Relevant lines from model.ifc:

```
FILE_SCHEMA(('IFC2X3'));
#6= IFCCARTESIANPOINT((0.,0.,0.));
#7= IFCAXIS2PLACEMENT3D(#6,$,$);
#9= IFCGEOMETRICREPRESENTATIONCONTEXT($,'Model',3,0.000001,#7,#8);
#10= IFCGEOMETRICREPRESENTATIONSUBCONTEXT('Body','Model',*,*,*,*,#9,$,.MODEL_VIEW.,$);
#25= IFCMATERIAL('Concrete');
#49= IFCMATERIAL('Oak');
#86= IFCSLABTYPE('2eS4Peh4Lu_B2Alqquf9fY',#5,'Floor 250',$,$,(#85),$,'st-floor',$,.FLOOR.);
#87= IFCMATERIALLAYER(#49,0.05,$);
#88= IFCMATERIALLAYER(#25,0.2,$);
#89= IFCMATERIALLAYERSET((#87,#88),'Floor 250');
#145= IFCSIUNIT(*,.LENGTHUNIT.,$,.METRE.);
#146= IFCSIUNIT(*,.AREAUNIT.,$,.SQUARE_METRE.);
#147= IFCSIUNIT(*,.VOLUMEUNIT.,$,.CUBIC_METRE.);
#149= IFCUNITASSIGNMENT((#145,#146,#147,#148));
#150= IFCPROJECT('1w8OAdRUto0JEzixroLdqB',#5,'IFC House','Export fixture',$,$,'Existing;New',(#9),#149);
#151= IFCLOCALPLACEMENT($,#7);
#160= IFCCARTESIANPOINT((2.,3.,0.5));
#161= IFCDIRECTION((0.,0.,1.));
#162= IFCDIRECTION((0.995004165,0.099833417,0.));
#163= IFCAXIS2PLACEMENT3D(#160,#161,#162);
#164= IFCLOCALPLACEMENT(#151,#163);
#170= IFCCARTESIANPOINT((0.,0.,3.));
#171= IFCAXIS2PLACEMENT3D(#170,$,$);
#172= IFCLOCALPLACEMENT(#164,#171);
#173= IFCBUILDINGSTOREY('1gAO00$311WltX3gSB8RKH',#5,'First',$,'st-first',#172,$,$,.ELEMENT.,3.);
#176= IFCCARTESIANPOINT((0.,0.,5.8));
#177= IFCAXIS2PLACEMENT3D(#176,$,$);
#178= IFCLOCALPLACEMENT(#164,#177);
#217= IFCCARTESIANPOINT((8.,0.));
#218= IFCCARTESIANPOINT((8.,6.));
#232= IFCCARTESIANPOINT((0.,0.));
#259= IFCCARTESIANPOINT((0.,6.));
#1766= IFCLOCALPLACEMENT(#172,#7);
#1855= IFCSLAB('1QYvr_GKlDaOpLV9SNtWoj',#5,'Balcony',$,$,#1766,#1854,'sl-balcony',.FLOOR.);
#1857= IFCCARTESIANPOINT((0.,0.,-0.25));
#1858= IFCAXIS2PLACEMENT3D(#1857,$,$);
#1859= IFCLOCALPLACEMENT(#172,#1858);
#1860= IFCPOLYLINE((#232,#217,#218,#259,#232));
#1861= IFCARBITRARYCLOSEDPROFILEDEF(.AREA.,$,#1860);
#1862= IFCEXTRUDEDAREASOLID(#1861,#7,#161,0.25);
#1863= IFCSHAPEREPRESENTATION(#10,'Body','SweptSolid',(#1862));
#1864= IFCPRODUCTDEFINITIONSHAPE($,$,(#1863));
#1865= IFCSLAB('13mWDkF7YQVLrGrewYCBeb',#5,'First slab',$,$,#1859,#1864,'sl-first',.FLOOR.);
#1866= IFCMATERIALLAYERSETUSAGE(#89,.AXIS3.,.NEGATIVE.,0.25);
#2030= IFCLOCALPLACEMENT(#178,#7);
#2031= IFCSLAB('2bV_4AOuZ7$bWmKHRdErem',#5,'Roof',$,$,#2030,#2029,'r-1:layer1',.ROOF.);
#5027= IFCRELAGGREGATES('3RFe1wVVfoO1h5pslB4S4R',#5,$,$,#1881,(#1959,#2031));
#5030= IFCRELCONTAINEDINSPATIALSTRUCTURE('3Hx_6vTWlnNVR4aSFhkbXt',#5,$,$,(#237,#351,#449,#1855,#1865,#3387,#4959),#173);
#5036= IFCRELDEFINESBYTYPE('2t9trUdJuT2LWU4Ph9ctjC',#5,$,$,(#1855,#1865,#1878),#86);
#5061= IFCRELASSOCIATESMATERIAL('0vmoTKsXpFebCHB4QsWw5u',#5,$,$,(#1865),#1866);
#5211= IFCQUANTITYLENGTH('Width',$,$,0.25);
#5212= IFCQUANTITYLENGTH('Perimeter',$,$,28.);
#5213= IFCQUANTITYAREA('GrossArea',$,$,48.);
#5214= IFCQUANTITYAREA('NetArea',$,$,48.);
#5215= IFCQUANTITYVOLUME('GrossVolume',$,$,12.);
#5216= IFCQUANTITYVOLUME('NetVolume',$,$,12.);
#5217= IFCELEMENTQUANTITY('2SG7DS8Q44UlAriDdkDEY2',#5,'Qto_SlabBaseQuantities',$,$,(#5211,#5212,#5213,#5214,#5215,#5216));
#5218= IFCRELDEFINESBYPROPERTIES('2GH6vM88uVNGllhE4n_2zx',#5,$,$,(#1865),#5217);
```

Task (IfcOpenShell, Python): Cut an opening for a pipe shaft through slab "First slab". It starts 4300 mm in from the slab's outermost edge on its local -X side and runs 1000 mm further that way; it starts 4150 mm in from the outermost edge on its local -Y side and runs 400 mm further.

```python
import numpy as np
import ifcopenshell
import ifcopenshell.api.feature
import ifcopenshell.api.geometry
import ifcopenshell.api.pset
import ifcopenshell.api.root
import ifcopenshell.geom
import ifcopenshell.util.element
import ifcopenshell.util.placement
import ifcopenshell.util.representation
import ifcopenshell.util.shape
import ifcopenshell.util.unit

model = ifcopenshell.open("model.ifc")
unit_scale = ifcopenshell.util.unit.calculate_unit_scale(model)
area_scale = ifcopenshell.util.unit.calculate_unit_scale(model, "AREAUNIT")
volume_scale = ifcopenshell.util.unit.calculate_unit_scale(model, "VOLUMEUNIT")
settings = ifcopenshell.geom.settings()


def volume(element):
    """Net volume in cubic metres, openings subtracted."""
    shape = ifcopenshell.geom.create_shape(settings, element)
    return ifcopenshell.util.shape.get_volume(shape.geometry)


slab = model.by_guid("13mWDkF7YQVLrGrewYCBeb")
before = volume(slab)

# Extent in the slab's own axes, in metres. The edges named are its -X and -Y sides.
slab_shape = ifcopenshell.geom.create_shape(settings, slab)
vertices = ifcopenshell.util.shape.get_vertices(slab_shape.geometry)
x_min, y_min, bottom = vertices.min(axis=0)
top = vertices[:, 2].max()

opening = ifcopenshell.api.root.create_entity(model, ifc_class="IfcOpeningElement", name="Pipe shaft opening")
context = ifcopenshell.util.representation.get_context(model, "Model", "Body", "MODEL_VIEW")
width, depth = 1, 0.4
outline = [(0.0, 0.0), (width, 0.0), (width, depth), (0.0, depth), (0.0, 0.0)]
# Overshoot both faces by 50 mm so the cut is clean.
shape = ifcopenshell.api.geometry.add_slab_representation(
    model, context=context, depth=top - bottom + 0.1, polyline=outline
)
ifcopenshell.api.geometry.assign_representation(model, product=opening, representation=shape)

matrix = ifcopenshell.util.placement.get_local_placement(slab.ObjectPlacement)
matrix[:, 3] = matrix @ np.append(np.array([x_min + 4.3, y_min + 4.15, bottom - 0.05]) / unit_scale, 1.0)
ifcopenshell.api.geometry.edit_object_placement(model, product=opening, matrix=matrix, is_si=False)
ifcopenshell.api.feature.add_feature(model, feature=opening, element=slab)

after = volume(slab)

# Update the slab's stored quantities.
qto = model.by_id(ifcopenshell.util.element.get_pset(slab, "Qto_SlabBaseQuantities", should_inherit=False)["id"])
ifcopenshell.api.pset.edit_qto(model, qto=qto, properties={
    "NetArea": after / (top - bottom) / area_scale,
    "NetVolume": after / volume_scale,
})

print(f"slab volume {before:.3f} -> {after:.3f} m3")

model.write("model_rev.ifc")
```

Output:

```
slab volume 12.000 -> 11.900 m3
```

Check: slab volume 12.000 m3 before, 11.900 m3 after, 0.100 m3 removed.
